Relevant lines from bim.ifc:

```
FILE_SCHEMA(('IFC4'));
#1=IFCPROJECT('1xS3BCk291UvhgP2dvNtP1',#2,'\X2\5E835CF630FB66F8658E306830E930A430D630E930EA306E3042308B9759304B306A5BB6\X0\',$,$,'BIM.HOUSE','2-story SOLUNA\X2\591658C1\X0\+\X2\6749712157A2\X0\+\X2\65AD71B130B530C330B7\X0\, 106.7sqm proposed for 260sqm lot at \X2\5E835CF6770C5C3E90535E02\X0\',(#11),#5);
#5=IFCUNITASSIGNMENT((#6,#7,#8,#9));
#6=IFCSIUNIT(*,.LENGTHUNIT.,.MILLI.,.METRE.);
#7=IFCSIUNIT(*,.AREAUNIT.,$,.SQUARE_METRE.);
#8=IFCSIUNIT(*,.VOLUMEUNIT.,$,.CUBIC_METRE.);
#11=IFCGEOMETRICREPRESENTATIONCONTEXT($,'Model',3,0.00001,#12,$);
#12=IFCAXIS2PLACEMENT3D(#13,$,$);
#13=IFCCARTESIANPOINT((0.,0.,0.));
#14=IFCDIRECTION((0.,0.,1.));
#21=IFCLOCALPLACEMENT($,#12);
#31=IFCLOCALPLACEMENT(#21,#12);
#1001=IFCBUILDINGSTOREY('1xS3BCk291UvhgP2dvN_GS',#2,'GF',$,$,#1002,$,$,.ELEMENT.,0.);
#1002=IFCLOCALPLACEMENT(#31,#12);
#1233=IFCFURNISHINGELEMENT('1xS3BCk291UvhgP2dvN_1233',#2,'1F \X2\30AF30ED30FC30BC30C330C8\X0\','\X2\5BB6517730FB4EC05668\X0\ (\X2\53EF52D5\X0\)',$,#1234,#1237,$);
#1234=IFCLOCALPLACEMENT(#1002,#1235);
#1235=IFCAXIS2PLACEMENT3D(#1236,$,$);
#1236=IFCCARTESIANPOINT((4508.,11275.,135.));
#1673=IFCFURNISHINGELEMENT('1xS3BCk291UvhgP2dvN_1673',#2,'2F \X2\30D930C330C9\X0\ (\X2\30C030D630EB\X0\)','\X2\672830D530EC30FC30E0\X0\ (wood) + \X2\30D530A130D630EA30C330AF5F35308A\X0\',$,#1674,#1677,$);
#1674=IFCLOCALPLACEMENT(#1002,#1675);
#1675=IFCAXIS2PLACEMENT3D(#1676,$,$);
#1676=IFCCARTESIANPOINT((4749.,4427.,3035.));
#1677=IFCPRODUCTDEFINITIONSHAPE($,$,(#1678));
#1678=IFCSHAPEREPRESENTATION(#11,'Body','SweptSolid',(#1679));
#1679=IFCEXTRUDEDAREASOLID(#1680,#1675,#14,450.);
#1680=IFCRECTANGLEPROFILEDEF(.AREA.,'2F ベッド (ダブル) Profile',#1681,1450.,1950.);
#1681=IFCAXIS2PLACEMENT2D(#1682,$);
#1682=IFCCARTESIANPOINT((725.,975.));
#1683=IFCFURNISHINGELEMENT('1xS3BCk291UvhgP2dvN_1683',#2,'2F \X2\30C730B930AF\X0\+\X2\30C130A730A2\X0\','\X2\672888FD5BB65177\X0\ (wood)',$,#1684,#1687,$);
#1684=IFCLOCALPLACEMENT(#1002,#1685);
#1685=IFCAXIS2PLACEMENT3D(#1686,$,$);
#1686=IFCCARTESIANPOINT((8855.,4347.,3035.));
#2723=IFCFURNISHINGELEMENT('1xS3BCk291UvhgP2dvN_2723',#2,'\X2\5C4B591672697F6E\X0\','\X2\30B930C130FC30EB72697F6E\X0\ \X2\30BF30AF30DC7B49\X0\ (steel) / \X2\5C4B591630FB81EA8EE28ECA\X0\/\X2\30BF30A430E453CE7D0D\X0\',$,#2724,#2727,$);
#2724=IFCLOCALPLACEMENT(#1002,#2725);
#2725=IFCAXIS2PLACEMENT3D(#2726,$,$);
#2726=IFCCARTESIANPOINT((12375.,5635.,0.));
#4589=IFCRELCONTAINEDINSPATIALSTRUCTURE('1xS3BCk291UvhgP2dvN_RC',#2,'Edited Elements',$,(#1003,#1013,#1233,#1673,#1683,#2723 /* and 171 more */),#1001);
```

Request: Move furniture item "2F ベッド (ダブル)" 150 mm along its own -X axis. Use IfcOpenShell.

```python
import ifcopenshell
import ifcopenshell.api.geometry
import ifcopenshell.util.placement

model = ifcopenshell.open("bim.ifc")

item = model.by_guid("1xS3BCk291UvhgP2dvN_1673")
matrix = ifcopenshell.util.placement.get_local_placement(item.ObjectPlacement)
matrix[:3, 3] -= matrix[:3, 0] * 150.0
ifcopenshell.api.geometry.edit_object_placement(model, product=item, matrix=matrix, is_si=False)

print(ifcopenshell.util.placement.get_local_placement(item.ObjectPlacement).round(3) + 0.0)

model.write("bim_updated.ifc")
```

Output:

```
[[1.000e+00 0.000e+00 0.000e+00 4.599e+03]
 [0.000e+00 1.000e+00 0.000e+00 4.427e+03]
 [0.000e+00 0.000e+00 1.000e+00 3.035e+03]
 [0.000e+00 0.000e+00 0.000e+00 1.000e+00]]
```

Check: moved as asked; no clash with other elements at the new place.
